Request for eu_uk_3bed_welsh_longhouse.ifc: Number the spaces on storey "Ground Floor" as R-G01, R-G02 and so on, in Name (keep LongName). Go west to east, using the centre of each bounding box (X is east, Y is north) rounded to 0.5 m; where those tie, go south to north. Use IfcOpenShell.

First a look at what the model holds.

```python
import ifcopenshell
import ifcopenshell.util.element
import ifcopenshell.util.placement

model = ifcopenshell.open("eu_uk_3bed_welsh_longhouse.ifc")
print(model.schema)
storey = next(s for s in model.by_type("IfcBuildingStorey") if s.Name == "Ground Floor")
spaces = [e for e in ifcopenshell.util.element.get_decomposition(storey) if e.is_a("IfcSpace")]
for e in sorted(spaces, key=lambda e: e.id()):
    origin = ifcopenshell.util.placement.get_local_placement(e.ObjectPlacement)[:3, 3]
    print(e.id(), e.Name, e.LongName, origin.round(2) + 0.0, sep=" | ")
```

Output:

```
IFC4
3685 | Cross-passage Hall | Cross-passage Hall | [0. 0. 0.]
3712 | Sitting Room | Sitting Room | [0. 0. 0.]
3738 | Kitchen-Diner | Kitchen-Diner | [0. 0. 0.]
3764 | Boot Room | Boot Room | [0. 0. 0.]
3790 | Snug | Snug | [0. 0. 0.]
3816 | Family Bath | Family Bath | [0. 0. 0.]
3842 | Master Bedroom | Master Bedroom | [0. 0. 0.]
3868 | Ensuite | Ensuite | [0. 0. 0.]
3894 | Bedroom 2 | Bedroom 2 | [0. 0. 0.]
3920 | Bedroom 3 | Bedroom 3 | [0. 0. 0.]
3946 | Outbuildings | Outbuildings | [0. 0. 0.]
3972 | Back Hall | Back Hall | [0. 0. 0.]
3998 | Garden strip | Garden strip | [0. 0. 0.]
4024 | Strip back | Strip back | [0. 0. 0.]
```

```python
import ifcopenshell
import ifcopenshell.geom
import ifcopenshell.util.element
import ifcopenshell.util.shape

model = ifcopenshell.open("eu_uk_3bed_welsh_longhouse.ifc")
settings = ifcopenshell.geom.settings()
settings.set("use-world-coords", True)


def centre(element):
    shape = ifcopenshell.geom.create_shape(settings, element)
    return ifcopenshell.util.shape.get_bbox_centroid(shape.geometry)


storey = next(s for s in model.by_type("IfcBuildingStorey") if s.Name == "Ground Floor")
spaces = [e for e in ifcopenshell.util.element.get_decomposition(storey) if e.is_a("IfcSpace")]

# Insertion points can sit at a corner or the storey origin, so sort by the geometry (in metres).
centres = {e: centre(e) for e in spaces}
spaces.sort(key=lambda e: (round(centres[e][0] / 0.5), centres[e][1]))

for i, e in enumerate(spaces, start=1):
    number = f"R-G{i:02d}"
    e.Name = number
    print(e.id(), number)

model.write("eu_uk_3bed_welsh_longhouse_rev.ifc")
```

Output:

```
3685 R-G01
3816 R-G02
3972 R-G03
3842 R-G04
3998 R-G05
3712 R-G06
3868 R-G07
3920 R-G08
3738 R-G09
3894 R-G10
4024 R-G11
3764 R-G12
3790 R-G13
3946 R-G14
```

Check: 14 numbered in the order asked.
